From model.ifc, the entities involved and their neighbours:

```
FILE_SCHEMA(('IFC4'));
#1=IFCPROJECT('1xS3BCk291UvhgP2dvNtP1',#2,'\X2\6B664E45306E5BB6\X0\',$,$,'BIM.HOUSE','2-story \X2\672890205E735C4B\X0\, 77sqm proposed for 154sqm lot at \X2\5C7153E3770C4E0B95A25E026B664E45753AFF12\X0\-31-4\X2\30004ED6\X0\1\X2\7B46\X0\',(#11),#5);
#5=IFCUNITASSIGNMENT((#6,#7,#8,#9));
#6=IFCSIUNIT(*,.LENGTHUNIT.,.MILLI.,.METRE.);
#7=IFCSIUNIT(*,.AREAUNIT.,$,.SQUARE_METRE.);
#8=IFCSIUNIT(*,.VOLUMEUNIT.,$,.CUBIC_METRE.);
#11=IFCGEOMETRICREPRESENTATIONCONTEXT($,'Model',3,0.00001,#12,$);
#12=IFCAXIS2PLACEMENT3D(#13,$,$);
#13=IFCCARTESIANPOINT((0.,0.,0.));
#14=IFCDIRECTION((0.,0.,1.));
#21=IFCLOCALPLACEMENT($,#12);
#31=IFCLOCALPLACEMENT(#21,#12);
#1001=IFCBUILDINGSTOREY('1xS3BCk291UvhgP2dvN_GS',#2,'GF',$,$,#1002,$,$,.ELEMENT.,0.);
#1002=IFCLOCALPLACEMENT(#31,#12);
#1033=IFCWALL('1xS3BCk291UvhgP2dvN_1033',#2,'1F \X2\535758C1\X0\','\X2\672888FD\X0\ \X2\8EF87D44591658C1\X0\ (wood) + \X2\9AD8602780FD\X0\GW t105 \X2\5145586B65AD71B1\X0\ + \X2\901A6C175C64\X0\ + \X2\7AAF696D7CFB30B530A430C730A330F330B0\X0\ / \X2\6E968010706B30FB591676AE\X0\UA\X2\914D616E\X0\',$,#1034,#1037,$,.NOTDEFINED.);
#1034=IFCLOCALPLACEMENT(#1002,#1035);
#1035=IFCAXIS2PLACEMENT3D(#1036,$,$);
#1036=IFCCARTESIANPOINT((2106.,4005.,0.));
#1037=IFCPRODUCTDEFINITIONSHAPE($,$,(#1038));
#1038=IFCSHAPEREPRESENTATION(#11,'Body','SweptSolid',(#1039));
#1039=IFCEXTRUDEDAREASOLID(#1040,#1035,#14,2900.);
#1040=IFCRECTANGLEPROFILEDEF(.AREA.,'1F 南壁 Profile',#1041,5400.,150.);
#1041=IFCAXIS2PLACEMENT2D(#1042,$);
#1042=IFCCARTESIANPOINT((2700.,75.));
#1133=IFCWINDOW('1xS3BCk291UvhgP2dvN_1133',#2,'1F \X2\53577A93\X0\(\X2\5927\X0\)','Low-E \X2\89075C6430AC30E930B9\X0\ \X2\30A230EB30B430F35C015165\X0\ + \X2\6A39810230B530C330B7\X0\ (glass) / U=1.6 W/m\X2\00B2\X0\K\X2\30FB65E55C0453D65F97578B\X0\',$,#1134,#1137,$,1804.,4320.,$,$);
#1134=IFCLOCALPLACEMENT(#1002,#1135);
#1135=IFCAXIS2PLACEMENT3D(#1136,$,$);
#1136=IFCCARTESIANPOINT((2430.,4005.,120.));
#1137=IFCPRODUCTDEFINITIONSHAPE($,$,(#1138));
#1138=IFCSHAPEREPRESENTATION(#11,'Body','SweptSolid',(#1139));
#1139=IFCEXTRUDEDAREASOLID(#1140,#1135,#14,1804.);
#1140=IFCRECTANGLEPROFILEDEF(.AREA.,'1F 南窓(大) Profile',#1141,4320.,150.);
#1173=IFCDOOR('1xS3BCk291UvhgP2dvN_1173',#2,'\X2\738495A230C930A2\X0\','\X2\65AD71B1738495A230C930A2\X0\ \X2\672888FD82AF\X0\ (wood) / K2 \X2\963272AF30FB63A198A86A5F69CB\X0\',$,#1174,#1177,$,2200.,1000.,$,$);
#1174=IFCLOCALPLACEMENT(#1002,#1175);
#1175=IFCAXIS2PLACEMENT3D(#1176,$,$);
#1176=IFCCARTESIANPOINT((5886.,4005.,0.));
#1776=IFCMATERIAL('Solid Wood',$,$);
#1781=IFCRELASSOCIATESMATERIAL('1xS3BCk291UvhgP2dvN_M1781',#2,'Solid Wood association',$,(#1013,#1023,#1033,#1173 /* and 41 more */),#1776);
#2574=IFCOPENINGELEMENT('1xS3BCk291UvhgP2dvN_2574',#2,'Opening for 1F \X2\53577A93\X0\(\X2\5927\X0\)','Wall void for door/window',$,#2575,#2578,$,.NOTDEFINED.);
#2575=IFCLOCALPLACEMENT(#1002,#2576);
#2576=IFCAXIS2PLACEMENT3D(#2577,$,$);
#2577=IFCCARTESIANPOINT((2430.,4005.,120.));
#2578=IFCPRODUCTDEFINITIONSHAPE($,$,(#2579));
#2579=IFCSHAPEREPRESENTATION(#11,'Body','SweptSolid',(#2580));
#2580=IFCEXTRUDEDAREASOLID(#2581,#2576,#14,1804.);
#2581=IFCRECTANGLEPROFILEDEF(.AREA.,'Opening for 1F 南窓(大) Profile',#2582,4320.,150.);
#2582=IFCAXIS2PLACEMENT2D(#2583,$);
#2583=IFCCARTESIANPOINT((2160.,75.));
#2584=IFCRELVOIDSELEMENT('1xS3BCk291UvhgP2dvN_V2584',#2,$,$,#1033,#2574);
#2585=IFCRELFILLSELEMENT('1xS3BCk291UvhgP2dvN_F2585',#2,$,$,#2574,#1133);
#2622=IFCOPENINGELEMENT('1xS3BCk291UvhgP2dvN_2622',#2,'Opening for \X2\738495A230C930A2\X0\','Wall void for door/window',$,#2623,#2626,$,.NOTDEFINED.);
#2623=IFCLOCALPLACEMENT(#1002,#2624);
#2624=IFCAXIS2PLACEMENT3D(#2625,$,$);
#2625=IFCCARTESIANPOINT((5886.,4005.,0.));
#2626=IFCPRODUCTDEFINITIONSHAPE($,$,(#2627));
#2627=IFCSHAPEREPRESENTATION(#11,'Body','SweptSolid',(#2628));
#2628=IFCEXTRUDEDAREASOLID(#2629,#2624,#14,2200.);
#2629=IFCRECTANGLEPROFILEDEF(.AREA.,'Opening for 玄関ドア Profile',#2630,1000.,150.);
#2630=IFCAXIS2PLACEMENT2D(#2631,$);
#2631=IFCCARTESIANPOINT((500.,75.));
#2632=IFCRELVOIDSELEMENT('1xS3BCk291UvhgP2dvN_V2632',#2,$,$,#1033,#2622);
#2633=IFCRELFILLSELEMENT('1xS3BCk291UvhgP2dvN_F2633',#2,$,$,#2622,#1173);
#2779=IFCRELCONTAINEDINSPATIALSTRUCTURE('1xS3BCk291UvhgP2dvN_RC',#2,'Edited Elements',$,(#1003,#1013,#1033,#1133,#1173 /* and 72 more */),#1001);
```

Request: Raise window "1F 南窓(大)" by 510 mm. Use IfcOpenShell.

```python
import numpy as np
import ifcopenshell
import ifcopenshell.api.geometry
import ifcopenshell.util.placement
import ifcopenshell.util.unit

model = ifcopenshell.open("model.ifc")
unit_scale = ifcopenshell.util.unit.calculate_unit_scale(model)

window = model.by_guid("1xS3BCk291UvhgP2dvN_1133")
opening = window.FillsVoids[0].RelatingOpeningElement
dz = 510.0

shift = np.array([0.0, 0.0, dz])
# The window is not placed relative to its opening, so move both.
for product in (opening, window):
    matrix = ifcopenshell.util.placement.get_local_placement(product.ObjectPlacement)
    matrix[:3, 3] += shift
    ifcopenshell.api.geometry.edit_object_placement(model, product=product, matrix=matrix, is_si=False)

print(f"moved by {dz * unit_scale:+.3f} m")

model.write("model_rev.ifc")
```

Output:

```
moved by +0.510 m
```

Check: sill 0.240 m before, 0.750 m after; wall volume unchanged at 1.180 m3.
